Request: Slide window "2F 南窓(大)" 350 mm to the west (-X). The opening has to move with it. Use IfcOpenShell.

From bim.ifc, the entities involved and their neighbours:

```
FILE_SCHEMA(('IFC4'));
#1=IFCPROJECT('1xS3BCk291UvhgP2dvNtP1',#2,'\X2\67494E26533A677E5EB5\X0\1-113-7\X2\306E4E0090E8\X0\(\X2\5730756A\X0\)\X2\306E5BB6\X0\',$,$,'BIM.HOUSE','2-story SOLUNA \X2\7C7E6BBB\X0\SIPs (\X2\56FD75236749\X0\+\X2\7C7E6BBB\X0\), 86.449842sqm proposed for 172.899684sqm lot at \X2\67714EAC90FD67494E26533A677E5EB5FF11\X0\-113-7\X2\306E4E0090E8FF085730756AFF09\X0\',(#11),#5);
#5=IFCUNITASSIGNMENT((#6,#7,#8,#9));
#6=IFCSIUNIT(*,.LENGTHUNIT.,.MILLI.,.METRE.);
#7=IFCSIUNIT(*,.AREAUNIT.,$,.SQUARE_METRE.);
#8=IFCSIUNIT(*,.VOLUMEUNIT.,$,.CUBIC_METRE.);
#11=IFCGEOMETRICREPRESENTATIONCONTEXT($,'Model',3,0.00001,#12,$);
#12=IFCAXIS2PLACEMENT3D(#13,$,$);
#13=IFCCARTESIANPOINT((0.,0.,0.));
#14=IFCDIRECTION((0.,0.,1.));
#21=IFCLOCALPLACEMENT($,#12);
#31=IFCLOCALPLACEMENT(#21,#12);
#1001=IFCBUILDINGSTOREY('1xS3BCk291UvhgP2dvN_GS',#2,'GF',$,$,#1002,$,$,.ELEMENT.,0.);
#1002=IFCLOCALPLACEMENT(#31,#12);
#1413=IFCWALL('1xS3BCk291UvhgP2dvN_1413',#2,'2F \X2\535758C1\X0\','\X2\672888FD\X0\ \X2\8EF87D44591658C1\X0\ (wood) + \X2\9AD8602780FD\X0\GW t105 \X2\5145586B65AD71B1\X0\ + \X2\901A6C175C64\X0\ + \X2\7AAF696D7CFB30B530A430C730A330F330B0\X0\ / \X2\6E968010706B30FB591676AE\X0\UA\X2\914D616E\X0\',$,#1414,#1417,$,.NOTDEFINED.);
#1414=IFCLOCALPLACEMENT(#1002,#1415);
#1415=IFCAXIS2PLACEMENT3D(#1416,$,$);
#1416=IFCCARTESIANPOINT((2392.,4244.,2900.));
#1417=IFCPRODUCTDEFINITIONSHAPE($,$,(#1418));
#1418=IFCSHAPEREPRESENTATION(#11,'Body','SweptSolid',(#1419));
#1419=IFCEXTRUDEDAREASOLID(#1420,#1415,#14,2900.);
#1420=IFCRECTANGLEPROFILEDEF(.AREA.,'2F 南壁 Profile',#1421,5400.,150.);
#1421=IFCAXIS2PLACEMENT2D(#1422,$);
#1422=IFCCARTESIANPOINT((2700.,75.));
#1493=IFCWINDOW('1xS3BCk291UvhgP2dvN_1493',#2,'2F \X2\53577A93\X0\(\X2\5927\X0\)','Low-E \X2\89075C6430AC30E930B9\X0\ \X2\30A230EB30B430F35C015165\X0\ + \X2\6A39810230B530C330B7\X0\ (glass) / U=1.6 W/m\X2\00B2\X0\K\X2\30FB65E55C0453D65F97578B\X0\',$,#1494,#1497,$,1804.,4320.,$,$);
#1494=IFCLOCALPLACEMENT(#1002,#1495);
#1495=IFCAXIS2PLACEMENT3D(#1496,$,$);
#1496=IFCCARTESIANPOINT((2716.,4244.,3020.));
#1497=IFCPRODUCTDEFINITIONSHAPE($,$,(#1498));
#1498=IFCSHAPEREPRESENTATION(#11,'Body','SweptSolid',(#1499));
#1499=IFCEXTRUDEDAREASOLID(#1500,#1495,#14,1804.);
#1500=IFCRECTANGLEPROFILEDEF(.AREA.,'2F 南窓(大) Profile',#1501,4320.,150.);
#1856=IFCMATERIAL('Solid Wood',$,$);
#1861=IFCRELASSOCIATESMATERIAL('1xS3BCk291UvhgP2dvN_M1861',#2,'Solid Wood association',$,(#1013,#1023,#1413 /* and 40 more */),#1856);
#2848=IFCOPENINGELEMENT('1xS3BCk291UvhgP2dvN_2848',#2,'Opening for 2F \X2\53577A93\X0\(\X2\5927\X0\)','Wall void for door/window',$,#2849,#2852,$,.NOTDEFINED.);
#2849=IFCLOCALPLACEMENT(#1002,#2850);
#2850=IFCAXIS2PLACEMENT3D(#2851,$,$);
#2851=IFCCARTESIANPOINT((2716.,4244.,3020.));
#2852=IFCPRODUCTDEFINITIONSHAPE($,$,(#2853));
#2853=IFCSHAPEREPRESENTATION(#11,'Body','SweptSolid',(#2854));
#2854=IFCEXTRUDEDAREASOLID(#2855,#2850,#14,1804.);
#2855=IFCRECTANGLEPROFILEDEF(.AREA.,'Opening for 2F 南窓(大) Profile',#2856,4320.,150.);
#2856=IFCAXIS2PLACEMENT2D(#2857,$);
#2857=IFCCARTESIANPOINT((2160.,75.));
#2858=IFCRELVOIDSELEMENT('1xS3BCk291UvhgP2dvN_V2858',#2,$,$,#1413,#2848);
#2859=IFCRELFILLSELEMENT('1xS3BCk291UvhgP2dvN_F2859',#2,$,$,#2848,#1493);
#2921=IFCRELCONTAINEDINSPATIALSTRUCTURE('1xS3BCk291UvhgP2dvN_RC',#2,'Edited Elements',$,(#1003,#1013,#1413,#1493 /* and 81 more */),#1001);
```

```python
import ifcopenshell
import ifcopenshell.api.geometry
import ifcopenshell.util.placement
import ifcopenshell.util.unit

model = ifcopenshell.open("bim.ifc")
unit_scale = ifcopenshell.util.unit.calculate_unit_scale(model)

window = model.by_guid("1xS3BCk291UvhgP2dvN_1493")
opening = window.FillsVoids[0].RelatingOpeningElement
wall = opening.VoidsElements[0].RelatingBuildingElement

wall_matrix = ifcopenshell.util.placement.get_local_placement(wall.ObjectPlacement)
shift = wall_matrix[:3, 0] * -0.35 / unit_scale
before = ifcopenshell.util.placement.get_local_placement(window.ObjectPlacement)[:3, 3].copy()

# The window is not placed relative to its opening, so move both.
for product in (opening, window):
    matrix = ifcopenshell.util.placement.get_local_placement(product.ObjectPlacement)
    matrix[:3, 3] += shift
    ifcopenshell.api.geometry.edit_object_placement(model, product=product, matrix=matrix, is_si=False)

after = ifcopenshell.util.placement.get_local_placement(window.ObjectPlacement)[:3, 3]
print("window moved by", (after - before).round(3) + 0.0)

model.write("bim_edited.ifc")
```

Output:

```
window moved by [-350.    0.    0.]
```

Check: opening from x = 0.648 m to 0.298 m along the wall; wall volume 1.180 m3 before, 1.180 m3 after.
